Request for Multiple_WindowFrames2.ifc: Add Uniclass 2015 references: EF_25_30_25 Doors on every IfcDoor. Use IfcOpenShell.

First a look at what the model holds.

```python
import ifcopenshell

model = ifcopenshell.open("Multiple_WindowFrames2.ifc")
print(model.schema)
print("classifications:", [c.Name for c in model.by_type("IfcClassification")])
for ifc_class in ("IfcDoor", "IfcRoof", "IfcStair", "IfcWall", "IfcWindow"):
    print(ifc_class, len(model.by_type(ifc_class)))
```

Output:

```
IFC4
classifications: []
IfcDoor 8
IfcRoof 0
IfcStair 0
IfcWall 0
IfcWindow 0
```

```python
import ifcopenshell
import ifcopenshell.api.classification

model = ifcopenshell.open("Multiple_WindowFrames2.ifc")

system = ifcopenshell.api.classification.add_classification(model, classification="Uniclass 2015")

codes = {
    "IfcDoor": ("EF_25_30_25", "Doors"),
}
for ifc_class, (code, name) in codes.items():
    products = model.by_type(ifc_class)
    ifcopenshell.api.classification.add_reference(
        model, products=products, classification=system, identification=code, name=name
    )
    print(code, len(products))

model.write("Multiple_WindowFrames2_v2.ifc")
```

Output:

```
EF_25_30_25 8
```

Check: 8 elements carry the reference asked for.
